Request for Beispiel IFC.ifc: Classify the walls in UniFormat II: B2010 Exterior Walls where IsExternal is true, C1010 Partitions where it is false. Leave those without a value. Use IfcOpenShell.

First a look at what the model holds.

```python
import ifcopenshell
import ifcopenshell.util.element

model = ifcopenshell.open("Beispiel IFC.ifc")
print(model.schema)
print("classifications:", [c.Name for c in model.by_type("IfcClassification")])
values = [ifcopenshell.util.element.get_pset(e, "Pset_WallCommon", "IsExternal") for e in model.by_type("IfcWall")]
for value in (True, False, None):
    print("IsExternal", value, values.count(value))
```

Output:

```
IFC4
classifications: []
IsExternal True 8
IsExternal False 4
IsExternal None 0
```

```python
import ifcopenshell
import ifcopenshell.api.classification
import ifcopenshell.util.element

model = ifcopenshell.open("Beispiel IFC.ifc")

system = ifcopenshell.api.classification.add_classification(model, classification="UniFormat II")

walls = model.by_type("IfcWall")
external = {e: ifcopenshell.util.element.get_pset(e, "Pset_WallCommon", "IsExternal") for e in walls}
for flag, code, name in ((True, "B2010", "Exterior Walls"), (False, "C1010", "Partitions")):
    products = [e for e in walls if external[e] is flag]
    ifcopenshell.api.classification.add_reference(
        model, products=products, classification=system, identification=code, name=name
    )
    print(code, len(products))

model.write("Beispiel IFC_edited.ifc")
```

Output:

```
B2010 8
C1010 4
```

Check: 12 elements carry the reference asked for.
